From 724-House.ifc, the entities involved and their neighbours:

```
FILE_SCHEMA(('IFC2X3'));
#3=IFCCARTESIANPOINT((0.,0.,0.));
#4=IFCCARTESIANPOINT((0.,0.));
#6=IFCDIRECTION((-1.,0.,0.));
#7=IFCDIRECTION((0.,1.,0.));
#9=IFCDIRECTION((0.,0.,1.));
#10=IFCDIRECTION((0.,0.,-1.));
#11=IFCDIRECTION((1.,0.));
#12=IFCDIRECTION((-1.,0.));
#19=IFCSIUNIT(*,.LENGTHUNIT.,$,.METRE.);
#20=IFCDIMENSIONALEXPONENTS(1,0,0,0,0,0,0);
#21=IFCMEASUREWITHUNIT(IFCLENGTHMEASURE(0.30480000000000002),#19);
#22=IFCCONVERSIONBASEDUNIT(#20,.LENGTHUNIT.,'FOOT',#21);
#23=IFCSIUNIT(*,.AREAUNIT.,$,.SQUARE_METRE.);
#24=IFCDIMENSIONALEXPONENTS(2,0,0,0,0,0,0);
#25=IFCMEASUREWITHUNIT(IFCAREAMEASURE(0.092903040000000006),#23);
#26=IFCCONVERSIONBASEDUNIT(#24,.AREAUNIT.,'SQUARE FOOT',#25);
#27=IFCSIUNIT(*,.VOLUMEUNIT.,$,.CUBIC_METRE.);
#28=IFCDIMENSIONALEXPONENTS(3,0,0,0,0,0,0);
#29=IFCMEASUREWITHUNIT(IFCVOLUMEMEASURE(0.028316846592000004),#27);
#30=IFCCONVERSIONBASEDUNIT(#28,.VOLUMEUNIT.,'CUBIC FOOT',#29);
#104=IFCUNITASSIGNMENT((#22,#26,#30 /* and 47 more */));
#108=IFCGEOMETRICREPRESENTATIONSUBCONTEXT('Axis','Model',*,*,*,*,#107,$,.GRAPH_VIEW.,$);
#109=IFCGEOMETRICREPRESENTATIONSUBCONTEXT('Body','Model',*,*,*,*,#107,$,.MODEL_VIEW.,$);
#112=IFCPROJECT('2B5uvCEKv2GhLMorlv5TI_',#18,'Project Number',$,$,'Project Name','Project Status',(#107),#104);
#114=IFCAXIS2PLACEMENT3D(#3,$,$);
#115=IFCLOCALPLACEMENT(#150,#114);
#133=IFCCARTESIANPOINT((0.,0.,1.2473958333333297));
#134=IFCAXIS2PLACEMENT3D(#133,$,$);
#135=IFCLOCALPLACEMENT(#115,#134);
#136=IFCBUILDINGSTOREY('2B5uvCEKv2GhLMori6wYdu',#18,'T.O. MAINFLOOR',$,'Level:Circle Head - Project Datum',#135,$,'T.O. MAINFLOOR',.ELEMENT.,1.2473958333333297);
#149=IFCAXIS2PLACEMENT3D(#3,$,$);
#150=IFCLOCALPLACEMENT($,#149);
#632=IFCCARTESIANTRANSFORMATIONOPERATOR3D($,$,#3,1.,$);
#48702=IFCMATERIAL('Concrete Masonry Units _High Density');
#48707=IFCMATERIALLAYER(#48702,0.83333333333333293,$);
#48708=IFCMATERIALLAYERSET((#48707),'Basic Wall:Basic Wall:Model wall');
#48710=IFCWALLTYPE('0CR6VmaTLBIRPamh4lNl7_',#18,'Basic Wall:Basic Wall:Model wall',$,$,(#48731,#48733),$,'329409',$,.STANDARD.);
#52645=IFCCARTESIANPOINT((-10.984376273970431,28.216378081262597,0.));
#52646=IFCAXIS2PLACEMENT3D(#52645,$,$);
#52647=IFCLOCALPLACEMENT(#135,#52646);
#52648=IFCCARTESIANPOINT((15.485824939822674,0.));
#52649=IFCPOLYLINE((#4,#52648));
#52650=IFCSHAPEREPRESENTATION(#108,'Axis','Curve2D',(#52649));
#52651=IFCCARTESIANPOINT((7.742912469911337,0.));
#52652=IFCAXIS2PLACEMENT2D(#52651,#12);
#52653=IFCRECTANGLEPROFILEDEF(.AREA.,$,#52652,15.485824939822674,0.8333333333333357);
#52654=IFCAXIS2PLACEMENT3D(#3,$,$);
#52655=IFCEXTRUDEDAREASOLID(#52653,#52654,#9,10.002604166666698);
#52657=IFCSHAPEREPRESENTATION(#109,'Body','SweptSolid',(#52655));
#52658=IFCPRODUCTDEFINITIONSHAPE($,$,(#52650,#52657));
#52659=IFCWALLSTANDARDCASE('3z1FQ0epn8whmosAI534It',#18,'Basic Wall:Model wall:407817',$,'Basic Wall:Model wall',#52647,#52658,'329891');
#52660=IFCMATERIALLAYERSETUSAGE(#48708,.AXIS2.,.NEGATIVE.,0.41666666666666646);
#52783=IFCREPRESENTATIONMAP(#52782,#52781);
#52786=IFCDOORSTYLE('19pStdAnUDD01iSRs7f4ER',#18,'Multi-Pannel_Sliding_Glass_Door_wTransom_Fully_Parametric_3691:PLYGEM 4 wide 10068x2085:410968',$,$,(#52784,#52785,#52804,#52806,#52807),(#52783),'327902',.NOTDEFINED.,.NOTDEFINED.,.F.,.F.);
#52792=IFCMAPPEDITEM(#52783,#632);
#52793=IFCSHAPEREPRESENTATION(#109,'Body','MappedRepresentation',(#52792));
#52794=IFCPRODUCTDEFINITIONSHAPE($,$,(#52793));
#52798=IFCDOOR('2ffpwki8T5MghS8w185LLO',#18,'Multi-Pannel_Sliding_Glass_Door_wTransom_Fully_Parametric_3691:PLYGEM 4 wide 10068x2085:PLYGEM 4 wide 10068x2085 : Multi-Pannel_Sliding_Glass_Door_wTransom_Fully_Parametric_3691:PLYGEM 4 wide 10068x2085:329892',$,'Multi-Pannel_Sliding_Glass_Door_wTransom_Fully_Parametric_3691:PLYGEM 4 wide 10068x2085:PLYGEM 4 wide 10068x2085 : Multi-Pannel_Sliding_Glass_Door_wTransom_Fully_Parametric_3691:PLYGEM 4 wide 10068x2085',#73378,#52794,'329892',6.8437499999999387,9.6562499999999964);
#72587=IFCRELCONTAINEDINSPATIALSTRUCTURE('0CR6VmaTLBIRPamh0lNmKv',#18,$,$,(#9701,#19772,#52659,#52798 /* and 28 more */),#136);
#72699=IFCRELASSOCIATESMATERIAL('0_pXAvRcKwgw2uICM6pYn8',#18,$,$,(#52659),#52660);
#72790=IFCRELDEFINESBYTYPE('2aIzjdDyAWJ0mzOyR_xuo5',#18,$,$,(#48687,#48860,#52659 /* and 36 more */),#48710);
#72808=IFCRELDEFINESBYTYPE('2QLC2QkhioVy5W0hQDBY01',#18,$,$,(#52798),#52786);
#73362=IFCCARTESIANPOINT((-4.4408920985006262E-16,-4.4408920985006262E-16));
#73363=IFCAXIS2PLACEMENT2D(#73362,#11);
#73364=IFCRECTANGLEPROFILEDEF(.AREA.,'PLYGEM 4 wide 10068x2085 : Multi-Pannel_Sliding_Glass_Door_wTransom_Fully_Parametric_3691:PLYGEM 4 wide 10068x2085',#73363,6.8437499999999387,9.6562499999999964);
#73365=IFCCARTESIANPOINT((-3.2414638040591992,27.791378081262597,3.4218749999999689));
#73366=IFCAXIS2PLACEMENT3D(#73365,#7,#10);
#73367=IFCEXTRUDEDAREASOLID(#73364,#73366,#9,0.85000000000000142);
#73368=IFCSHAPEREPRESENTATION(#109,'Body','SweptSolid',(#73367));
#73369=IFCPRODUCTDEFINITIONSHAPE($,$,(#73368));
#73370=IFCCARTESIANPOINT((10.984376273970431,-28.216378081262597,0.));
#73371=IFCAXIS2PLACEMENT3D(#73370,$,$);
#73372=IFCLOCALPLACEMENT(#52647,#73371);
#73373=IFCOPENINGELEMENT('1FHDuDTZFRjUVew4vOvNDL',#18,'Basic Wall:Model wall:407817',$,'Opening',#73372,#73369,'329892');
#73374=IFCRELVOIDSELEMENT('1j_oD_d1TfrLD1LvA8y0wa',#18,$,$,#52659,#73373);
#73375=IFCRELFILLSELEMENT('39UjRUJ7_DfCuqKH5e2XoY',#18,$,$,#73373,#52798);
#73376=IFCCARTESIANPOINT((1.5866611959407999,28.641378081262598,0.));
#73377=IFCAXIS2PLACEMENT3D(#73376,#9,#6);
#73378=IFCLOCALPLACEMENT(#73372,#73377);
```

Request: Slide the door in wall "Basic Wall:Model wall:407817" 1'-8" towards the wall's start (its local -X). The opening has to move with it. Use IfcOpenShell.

```python
import ifcopenshell
import ifcopenshell.api.geometry
import ifcopenshell.util.placement
import ifcopenshell.util.unit

model = ifcopenshell.open("724-House.ifc")
unit_scale = ifcopenshell.util.unit.calculate_unit_scale(model)

door = model.by_id(52798)
opening = door.FillsVoids[0].RelatingOpeningElement
wall = opening.VoidsElements[0].RelatingBuildingElement

wall_matrix = ifcopenshell.util.placement.get_local_placement(wall.ObjectPlacement)
shift = wall_matrix[:3, 0] * -20 * 0.0254 / unit_scale
before = ifcopenshell.util.placement.get_local_placement(door.ObjectPlacement)[:3, 3].copy()

# The door is placed relative to its opening, so it follows when the opening moves.
matrix = ifcopenshell.util.placement.get_local_placement(opening.ObjectPlacement)
matrix[:3, 3] += shift
ifcopenshell.api.geometry.edit_object_placement(
    model, product=opening, matrix=matrix, is_si=False, should_transform_children=True
)

after = ifcopenshell.util.placement.get_local_placement(door.ObjectPlacement)[:3, 3]
print("door moved by", (after - before).round(3) + 0.0)

model.write("724-House_v2.ifc")
```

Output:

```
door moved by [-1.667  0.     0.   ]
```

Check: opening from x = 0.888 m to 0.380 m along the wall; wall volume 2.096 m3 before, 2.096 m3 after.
